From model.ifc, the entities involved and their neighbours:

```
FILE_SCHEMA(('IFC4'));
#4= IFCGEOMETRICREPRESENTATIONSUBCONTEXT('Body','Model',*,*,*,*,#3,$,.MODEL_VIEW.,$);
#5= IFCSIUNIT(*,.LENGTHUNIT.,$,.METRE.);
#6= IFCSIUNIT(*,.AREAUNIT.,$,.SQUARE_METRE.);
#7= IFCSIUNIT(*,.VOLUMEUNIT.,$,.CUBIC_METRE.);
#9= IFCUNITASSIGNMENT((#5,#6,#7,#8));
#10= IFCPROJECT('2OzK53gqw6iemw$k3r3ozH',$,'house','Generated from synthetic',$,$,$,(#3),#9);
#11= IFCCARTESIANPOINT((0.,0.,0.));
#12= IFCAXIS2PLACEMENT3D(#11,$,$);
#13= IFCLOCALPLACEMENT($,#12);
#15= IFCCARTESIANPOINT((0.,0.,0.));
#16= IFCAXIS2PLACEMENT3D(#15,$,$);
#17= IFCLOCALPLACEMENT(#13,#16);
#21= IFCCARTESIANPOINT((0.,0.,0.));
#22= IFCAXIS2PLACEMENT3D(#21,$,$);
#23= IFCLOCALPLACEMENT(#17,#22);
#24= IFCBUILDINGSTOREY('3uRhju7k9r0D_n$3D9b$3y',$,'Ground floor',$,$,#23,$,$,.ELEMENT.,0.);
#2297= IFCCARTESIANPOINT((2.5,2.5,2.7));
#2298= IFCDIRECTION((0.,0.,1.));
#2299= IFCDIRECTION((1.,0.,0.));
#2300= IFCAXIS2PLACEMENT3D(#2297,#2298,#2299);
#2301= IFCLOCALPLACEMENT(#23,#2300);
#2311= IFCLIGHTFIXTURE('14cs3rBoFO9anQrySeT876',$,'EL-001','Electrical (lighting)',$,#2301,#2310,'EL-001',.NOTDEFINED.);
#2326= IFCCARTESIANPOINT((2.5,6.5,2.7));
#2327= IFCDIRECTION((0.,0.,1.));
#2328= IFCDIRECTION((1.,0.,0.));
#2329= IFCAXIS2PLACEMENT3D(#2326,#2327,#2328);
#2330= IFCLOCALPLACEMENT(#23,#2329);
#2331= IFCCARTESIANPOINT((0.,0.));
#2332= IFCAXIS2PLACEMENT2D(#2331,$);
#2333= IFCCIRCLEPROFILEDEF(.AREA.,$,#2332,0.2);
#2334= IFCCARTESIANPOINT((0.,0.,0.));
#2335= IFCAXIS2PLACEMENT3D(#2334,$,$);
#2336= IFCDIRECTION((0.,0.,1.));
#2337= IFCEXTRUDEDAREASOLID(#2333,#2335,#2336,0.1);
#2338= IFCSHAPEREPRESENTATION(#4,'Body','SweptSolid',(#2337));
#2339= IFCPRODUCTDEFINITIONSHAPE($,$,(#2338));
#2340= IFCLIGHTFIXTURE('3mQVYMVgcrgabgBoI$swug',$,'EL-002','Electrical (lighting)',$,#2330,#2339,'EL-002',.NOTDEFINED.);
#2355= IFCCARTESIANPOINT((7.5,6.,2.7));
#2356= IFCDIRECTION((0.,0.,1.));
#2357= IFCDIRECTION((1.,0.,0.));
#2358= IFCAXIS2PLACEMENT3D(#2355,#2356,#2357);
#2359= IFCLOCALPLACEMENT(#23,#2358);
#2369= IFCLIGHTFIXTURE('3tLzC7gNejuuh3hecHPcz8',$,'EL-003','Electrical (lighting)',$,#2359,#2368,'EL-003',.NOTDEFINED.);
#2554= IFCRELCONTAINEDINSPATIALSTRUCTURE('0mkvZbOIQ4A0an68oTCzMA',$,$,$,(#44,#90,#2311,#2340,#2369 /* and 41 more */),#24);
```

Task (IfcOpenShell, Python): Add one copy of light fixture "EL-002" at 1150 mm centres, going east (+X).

```python
import numpy as np
import ifcopenshell
import ifcopenshell.api.geometry
import ifcopenshell.api.root
import ifcopenshell.util.element
import ifcopenshell.util.placement

model = ifcopenshell.open("model.ifc")

source = model.by_guid("3mQVYMVgcrgabgBoI$swug")
base = ifcopenshell.util.placement.get_local_placement(source.ObjectPlacement)
step = np.array([1.0, 0.0, 0.0]) * 1.15

for i in range(1, 2):
    copy = ifcopenshell.api.root.copy_class(model, product=source)
    copy.Representation = ifcopenshell.util.element.copy_deep(
        model, source.Representation, exclude=["IfcGeometricRepresentationContext", "IfcRepresentationMap"]
    )
    copy.Tag = None
    matrix = base.copy()
    matrix[:3, 3] += i * step
    print("added at", matrix[:3, 3].round(3) + 0.0)
    ifcopenshell.api.geometry.edit_object_placement(model, product=copy, matrix=matrix, is_si=False)

model.write("model_rev.ifc")
```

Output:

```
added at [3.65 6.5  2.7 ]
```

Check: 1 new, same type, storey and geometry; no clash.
